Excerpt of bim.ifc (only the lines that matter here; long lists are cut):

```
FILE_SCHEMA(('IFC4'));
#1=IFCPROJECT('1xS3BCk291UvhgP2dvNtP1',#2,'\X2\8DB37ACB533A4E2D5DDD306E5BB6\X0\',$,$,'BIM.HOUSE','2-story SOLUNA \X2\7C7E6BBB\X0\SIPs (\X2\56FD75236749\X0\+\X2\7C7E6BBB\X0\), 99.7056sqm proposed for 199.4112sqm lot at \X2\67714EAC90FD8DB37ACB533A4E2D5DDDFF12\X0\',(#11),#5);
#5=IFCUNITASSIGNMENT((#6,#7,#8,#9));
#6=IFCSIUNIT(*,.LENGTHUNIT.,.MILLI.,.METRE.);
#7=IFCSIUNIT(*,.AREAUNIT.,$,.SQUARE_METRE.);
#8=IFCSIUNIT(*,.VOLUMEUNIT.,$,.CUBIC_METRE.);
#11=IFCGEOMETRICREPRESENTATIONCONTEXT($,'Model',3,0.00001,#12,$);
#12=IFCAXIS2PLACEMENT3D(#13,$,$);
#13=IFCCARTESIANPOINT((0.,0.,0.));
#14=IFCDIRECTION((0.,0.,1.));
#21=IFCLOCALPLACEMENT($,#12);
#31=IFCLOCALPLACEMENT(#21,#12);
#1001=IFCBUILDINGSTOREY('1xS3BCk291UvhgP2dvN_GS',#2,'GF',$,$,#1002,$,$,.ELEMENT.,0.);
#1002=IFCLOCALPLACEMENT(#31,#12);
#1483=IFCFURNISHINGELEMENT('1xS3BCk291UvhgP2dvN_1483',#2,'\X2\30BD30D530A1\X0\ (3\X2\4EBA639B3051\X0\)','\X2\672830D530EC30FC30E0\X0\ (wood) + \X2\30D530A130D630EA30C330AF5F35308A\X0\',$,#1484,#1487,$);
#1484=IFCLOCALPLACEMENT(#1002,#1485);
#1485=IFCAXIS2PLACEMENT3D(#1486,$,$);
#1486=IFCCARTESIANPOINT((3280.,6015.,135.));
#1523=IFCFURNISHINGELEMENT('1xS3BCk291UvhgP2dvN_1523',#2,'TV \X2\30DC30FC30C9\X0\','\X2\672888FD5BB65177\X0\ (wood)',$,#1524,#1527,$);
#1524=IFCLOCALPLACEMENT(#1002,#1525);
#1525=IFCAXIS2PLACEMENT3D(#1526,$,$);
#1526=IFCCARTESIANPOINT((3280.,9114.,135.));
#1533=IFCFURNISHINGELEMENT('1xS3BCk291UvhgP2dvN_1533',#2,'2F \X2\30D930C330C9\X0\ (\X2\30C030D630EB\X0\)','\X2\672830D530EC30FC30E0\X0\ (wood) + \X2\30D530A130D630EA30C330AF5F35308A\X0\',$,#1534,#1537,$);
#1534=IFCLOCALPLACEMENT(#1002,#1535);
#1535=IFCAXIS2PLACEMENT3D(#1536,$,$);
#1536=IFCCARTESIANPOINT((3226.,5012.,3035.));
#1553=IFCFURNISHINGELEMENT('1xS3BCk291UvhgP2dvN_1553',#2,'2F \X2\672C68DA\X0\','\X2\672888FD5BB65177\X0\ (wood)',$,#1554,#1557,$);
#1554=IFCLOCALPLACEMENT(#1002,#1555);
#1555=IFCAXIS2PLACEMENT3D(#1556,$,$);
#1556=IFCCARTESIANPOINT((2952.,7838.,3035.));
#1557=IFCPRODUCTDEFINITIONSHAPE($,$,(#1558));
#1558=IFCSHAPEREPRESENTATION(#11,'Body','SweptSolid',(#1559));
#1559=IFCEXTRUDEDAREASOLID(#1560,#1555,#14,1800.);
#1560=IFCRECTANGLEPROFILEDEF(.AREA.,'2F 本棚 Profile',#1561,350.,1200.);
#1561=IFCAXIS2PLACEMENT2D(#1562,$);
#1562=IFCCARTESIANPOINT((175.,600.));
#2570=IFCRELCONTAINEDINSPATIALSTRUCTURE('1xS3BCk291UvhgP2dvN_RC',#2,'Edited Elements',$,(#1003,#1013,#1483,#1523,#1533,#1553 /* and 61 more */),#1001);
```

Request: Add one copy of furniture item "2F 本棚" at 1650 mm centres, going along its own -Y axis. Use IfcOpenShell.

```python
import ifcopenshell
import ifcopenshell.api.geometry
import ifcopenshell.api.root
import ifcopenshell.util.element
import ifcopenshell.util.placement

model = ifcopenshell.open("bim.ifc")


def reuse_history(source, copy):
    """copy_class also copies each property set's owner history, people and application; keep the originals."""
    for rel in copy.IsDefinedBy:
        if rel.is_a("IfcRelDefinesByProperties") and (history := rel.RelatingPropertyDefinition.OwnerHistory):
            rel.RelatingPropertyDefinition.OwnerHistory = source.OwnerHistory
            ifcopenshell.util.element.remove_deep2(model, history)


source = model.by_guid("1xS3BCk291UvhgP2dvN_1553")
base = ifcopenshell.util.placement.get_local_placement(source.ObjectPlacement)
step = -base[:3, 1] * 1650.0

for i in range(1, 2):
    copy = ifcopenshell.api.root.copy_class(model, product=source)
    copy.Representation = ifcopenshell.util.element.copy_deep(
        model, source.Representation, exclude=["IfcGeometricRepresentationContext", "IfcRepresentationMap"]
    )
    reuse_history(source, copy)
    matrix = base.copy()
    matrix[:3, 3] += i * step
    print("added at", matrix[:3, 3].round(3) + 0.0)
    ifcopenshell.api.geometry.edit_object_placement(model, product=copy, matrix=matrix, is_si=False)

model.write("bim_updated.ifc")
```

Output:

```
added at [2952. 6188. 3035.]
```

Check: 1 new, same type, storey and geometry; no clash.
